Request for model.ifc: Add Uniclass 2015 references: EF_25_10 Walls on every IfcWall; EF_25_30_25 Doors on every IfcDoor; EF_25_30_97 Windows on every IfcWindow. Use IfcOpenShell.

First a look at what the model holds.

```python
import ifcopenshell

model = ifcopenshell.open("model.ifc")
print(model.schema)
print("classifications:", [c.Name for c in model.by_type("IfcClassification")])
for ifc_class in ("IfcDoor", "IfcRoof", "IfcStair", "IfcWall", "IfcWindow"):
    print(ifc_class, len(model.by_type(ifc_class)))
```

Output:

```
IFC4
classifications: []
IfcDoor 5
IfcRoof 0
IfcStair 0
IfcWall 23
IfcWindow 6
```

```python
import ifcopenshell
import ifcopenshell.api.classification

model = ifcopenshell.open("model.ifc")

system = ifcopenshell.api.classification.add_classification(model, classification="Uniclass 2015")

codes = {
    "IfcWall": ("EF_25_10", "Walls"),
    "IfcDoor": ("EF_25_30_25", "Doors"),
    "IfcWindow": ("EF_25_30_97", "Windows"),
}
for ifc_class, (code, name) in codes.items():
    products = model.by_type(ifc_class)
    ifcopenshell.api.classification.add_reference(
        model, products=products, classification=system, identification=code, name=name
    )
    print(code, len(products))

model.write("model_edited.ifc")
```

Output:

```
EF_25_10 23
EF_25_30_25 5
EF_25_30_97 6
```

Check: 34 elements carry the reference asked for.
